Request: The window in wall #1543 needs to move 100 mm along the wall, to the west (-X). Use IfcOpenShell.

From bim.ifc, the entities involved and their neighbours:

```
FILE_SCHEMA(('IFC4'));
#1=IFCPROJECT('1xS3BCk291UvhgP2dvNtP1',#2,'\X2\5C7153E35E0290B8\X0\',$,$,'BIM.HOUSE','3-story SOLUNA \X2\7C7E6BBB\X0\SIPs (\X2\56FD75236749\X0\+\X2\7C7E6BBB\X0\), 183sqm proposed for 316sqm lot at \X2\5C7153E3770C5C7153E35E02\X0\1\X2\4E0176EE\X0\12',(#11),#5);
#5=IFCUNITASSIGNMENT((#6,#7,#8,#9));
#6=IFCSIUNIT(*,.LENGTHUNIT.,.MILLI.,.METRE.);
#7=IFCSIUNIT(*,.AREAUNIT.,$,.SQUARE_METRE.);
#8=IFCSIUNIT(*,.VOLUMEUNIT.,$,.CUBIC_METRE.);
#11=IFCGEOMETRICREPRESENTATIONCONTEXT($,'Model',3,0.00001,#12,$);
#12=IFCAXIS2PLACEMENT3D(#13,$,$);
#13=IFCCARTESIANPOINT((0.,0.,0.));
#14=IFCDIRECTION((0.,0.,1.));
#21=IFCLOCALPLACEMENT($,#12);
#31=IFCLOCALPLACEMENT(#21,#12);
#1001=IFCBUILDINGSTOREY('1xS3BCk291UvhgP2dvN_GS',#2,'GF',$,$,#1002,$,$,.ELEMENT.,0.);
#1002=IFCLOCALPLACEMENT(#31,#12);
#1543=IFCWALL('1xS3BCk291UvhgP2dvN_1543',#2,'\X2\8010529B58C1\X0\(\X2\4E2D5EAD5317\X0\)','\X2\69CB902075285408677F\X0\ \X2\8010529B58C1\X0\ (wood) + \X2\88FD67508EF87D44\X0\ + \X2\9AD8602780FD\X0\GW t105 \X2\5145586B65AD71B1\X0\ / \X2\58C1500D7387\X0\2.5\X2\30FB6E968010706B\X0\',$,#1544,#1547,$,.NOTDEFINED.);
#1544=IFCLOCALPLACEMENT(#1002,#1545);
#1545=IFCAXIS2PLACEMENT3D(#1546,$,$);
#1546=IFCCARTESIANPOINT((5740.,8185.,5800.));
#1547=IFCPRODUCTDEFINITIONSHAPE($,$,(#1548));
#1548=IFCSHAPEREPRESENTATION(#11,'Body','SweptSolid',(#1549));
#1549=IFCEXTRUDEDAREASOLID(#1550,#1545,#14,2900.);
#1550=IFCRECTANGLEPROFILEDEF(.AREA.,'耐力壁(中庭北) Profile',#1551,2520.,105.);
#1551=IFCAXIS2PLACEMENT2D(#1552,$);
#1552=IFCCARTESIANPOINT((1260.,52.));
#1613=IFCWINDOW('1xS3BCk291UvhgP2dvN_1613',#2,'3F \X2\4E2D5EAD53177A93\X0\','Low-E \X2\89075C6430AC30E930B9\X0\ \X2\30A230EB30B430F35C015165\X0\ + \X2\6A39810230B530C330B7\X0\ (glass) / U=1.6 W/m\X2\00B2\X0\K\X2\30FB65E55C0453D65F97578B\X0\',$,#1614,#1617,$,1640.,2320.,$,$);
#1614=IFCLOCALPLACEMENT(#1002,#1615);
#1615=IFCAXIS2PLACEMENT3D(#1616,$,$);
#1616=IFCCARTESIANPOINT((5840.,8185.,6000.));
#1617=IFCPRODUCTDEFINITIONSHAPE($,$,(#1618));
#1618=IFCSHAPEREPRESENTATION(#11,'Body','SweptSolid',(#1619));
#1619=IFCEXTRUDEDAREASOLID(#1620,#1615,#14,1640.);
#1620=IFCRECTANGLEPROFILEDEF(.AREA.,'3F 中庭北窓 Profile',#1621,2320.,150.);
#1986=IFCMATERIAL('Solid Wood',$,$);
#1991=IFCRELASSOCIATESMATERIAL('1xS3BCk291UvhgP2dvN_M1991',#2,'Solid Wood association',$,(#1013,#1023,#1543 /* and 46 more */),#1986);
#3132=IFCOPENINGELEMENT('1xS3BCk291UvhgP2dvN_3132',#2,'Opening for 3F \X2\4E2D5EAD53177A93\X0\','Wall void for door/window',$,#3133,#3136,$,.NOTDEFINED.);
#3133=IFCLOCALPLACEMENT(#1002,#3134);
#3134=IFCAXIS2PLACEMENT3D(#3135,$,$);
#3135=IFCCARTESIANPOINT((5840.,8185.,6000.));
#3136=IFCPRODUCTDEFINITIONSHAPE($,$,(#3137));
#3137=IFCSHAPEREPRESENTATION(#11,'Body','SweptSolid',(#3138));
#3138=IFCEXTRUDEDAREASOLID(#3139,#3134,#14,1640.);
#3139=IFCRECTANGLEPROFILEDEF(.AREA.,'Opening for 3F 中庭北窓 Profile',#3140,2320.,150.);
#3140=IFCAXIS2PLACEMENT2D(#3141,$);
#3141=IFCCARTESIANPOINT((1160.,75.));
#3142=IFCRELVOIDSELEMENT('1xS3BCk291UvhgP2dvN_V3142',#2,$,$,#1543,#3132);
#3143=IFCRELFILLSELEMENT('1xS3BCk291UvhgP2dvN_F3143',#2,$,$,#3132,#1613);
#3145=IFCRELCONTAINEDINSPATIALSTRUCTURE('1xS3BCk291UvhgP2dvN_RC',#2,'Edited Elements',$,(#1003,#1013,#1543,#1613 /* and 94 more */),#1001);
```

```python
import ifcopenshell
import ifcopenshell.api.geometry
import ifcopenshell.util.placement
import ifcopenshell.util.unit

model = ifcopenshell.open("bim.ifc")
unit_scale = ifcopenshell.util.unit.calculate_unit_scale(model)

window = model.by_guid("1xS3BCk291UvhgP2dvN_1613")
opening = window.FillsVoids[0].RelatingOpeningElement
wall = opening.VoidsElements[0].RelatingBuildingElement

wall_matrix = ifcopenshell.util.placement.get_local_placement(wall.ObjectPlacement)
shift = wall_matrix[:3, 0] * -0.1 / unit_scale
before = ifcopenshell.util.placement.get_local_placement(window.ObjectPlacement)[:3, 3].copy()

# The window is not placed relative to its opening, so move both.
for product in (opening, window):
    matrix = ifcopenshell.util.placement.get_local_placement(product.ObjectPlacement)
    matrix[:3, 3] += shift
    ifcopenshell.api.geometry.edit_object_placement(model, product=product, matrix=matrix, is_si=False)

after = ifcopenshell.util.placement.get_local_placement(window.ObjectPlacement)[:3, 3]
print("window moved by", (after - before).round(3) + 0.0)

model.write("bim_rev.ifc")
```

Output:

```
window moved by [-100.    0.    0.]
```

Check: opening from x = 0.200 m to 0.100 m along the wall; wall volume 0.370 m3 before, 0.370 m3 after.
